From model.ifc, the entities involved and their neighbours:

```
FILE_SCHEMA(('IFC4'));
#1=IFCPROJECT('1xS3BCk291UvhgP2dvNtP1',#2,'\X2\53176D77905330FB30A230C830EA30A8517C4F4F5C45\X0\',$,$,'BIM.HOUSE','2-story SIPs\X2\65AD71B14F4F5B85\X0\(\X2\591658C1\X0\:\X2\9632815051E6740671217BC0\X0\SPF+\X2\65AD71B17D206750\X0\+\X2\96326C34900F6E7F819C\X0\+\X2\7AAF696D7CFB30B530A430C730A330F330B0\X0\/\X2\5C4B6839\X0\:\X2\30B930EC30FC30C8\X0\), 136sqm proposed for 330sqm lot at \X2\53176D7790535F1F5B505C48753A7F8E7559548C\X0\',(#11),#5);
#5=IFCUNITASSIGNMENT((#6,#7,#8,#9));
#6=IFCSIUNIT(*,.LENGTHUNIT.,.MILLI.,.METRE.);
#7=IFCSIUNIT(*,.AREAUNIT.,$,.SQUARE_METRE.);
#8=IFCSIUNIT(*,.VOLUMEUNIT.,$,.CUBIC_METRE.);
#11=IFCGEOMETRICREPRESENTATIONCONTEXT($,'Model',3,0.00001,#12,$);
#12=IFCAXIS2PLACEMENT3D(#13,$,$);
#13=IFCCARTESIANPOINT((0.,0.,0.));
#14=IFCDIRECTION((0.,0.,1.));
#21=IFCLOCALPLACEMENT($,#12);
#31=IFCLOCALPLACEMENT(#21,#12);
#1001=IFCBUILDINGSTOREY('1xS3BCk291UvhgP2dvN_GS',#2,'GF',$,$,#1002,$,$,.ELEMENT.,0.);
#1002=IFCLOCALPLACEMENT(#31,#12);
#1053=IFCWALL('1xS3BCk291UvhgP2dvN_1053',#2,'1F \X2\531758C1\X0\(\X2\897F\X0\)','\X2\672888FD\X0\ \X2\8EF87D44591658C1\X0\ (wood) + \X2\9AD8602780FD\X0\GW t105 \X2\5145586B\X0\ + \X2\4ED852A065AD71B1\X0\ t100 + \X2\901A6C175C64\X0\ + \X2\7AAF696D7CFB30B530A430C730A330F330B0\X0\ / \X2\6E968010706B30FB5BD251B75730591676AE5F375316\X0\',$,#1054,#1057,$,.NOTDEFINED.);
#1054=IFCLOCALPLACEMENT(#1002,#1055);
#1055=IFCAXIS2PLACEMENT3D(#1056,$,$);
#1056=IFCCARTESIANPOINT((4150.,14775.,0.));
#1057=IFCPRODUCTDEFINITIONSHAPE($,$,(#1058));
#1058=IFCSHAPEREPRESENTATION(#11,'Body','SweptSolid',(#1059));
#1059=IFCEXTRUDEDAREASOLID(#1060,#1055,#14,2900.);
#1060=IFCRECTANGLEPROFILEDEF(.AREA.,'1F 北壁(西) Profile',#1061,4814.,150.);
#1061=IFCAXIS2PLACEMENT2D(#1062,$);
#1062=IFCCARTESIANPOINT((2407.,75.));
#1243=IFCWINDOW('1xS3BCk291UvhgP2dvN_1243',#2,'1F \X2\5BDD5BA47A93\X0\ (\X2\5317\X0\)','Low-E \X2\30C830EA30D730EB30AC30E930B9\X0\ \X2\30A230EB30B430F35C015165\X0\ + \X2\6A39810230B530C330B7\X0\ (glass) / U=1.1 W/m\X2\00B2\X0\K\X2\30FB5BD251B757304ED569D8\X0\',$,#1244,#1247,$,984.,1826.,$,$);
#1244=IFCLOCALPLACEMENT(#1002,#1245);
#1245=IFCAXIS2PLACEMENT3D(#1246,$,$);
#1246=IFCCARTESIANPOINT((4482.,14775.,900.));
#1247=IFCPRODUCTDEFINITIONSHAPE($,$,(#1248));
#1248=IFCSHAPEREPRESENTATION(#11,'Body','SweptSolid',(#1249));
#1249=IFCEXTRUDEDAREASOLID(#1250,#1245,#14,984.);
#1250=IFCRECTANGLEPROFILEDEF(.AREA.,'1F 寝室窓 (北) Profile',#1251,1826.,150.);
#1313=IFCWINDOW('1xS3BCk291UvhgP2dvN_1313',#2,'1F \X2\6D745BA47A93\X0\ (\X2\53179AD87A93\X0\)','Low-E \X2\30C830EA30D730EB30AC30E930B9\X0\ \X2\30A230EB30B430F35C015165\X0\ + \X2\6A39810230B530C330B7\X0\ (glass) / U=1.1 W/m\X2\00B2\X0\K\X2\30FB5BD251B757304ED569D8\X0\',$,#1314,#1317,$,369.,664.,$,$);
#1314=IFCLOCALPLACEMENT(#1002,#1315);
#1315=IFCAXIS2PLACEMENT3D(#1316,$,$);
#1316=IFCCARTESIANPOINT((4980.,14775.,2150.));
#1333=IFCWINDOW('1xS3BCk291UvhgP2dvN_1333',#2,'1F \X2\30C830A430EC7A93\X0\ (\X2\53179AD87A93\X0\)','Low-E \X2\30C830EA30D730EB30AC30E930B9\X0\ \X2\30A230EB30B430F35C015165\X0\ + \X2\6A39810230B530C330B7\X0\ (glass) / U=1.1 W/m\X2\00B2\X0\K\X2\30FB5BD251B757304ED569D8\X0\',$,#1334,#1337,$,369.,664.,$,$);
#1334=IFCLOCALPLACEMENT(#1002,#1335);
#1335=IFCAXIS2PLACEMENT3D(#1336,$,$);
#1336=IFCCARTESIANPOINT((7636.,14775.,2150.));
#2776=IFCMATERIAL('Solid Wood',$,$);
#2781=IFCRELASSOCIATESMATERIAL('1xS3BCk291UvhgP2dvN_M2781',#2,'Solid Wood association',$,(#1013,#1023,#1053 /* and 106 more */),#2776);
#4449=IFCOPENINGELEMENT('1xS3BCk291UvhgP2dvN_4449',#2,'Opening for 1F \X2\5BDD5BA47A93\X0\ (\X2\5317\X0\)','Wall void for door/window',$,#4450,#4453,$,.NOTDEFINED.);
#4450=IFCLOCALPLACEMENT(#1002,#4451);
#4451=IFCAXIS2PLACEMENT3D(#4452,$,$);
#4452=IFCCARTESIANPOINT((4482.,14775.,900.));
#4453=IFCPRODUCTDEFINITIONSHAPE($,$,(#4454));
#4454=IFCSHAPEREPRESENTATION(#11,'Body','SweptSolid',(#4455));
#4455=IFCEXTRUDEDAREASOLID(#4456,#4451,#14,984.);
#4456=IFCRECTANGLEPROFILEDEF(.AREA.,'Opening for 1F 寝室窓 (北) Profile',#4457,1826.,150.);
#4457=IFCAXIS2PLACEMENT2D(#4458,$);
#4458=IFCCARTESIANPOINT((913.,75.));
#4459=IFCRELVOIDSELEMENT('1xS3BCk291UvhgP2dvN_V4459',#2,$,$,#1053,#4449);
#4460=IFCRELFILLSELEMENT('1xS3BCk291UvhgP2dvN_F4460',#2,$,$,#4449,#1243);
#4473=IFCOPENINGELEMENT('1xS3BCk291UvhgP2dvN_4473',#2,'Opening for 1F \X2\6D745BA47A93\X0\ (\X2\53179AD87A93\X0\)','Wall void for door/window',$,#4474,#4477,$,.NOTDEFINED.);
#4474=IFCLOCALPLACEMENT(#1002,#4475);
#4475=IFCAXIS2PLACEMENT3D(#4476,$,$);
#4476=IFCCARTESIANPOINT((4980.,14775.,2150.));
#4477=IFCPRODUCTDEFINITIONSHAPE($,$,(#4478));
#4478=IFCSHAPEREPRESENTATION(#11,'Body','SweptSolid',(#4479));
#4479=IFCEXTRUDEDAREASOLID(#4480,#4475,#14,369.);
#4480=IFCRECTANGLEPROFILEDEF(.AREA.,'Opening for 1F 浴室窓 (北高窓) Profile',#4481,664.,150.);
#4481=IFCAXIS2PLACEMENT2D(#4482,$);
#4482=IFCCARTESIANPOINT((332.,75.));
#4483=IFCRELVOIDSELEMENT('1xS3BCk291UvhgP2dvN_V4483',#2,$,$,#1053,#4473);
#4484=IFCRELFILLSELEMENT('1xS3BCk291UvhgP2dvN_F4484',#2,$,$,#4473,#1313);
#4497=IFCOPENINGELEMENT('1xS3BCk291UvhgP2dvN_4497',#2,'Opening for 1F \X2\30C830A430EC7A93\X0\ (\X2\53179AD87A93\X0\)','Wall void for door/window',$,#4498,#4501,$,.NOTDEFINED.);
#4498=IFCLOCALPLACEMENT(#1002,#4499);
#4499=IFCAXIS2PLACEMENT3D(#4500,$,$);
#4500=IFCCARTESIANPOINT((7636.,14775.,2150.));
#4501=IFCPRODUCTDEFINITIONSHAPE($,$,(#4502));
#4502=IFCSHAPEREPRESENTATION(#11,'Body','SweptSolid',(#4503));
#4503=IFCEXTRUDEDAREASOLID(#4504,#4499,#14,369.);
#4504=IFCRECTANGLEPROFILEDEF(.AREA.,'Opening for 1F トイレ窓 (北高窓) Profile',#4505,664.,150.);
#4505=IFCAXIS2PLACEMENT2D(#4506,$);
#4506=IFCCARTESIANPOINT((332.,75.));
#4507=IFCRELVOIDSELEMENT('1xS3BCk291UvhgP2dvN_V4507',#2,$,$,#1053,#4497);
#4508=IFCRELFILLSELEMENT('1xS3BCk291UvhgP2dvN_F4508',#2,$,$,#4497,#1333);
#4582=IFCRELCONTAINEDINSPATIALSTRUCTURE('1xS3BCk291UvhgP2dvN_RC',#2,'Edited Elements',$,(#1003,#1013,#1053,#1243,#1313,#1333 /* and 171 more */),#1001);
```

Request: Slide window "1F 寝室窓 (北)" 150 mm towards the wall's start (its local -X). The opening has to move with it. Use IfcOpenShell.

```python
import ifcopenshell
import ifcopenshell.api.geometry
import ifcopenshell.util.placement

model = ifcopenshell.open("model.ifc")

window = model.by_guid("1xS3BCk291UvhgP2dvN_1243")
opening = window.FillsVoids[0].RelatingOpeningElement
wall = opening.VoidsElements[0].RelatingBuildingElement

wall_matrix = ifcopenshell.util.placement.get_local_placement(wall.ObjectPlacement)
shift = wall_matrix[:3, 0] * -150.0
before = ifcopenshell.util.placement.get_local_placement(window.ObjectPlacement)[:3, 3].copy()

# The window is not placed relative to its opening, so move both.
for product in (opening, window):
    matrix = ifcopenshell.util.placement.get_local_placement(product.ObjectPlacement)
    matrix[:3, 3] += shift
    ifcopenshell.api.geometry.edit_object_placement(model, product=product, matrix=matrix, is_si=False)

after = ifcopenshell.util.placement.get_local_placement(window.ObjectPlacement)[:3, 3]
print("window moved by", (after - before).round(3) + 0.0)

model.write("model_v2.ifc")
```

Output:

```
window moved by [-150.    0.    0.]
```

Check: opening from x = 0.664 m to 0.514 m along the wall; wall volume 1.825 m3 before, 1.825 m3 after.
